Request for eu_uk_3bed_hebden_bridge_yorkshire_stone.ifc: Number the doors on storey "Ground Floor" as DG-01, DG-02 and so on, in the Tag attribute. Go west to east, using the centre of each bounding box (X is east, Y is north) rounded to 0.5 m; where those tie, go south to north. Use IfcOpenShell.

First a look at what the model holds.

```python
import ifcopenshell
import ifcopenshell.util.element
import ifcopenshell.util.placement

model = ifcopenshell.open("eu_uk_3bed_hebden_bridge_yorkshire_stone.ifc")
print(model.schema)
storey = next(s for s in model.by_type("IfcBuildingStorey") if s.Name == "Ground Floor")
doors = [e for e in ifcopenshell.util.element.get_decomposition(storey) if e.is_a("IfcDoor")]
for e in sorted(doors, key=lambda e: e.id()):
    origin = ifcopenshell.util.placement.get_local_placement(e.ObjectPlacement)[:3, 3]
    print(e.id(), e.Tag, e.Name, origin.round(2) + 0.0, sep=" | ")
```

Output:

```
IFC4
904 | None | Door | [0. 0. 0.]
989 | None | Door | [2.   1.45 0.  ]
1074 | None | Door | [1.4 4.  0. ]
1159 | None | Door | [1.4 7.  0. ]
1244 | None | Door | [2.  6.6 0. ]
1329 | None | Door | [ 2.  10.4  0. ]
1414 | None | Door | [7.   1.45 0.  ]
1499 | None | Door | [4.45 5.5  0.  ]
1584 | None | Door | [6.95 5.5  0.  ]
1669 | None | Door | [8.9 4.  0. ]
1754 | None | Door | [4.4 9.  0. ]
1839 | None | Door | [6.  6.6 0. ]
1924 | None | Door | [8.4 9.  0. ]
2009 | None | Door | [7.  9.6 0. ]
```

```python
import ifcopenshell
import ifcopenshell.geom
import ifcopenshell.util.element
import ifcopenshell.util.shape

model = ifcopenshell.open("eu_uk_3bed_hebden_bridge_yorkshire_stone.ifc")
settings = ifcopenshell.geom.settings()
settings.set("use-world-coords", True)


def centre(element):
    shape = ifcopenshell.geom.create_shape(settings, element)
    return ifcopenshell.util.shape.get_bbox_centroid(shape.geometry)


storey = next(s for s in model.by_type("IfcBuildingStorey") if s.Name == "Ground Floor")
doors = [e for e in ifcopenshell.util.element.get_decomposition(storey) if e.is_a("IfcDoor")]

# Insertion points can sit at a corner or the storey origin, so sort by the geometry (in metres).
centres = {e: centre(e) for e in doors}
doors.sort(key=lambda e: (round(centres[e][0] / 0.5), centres[e][1]))

for i, e in enumerate(doors, start=1):
    number = f"DG-{i:02d}"
    e.Tag = number
    print(e.id(), number)

model.write("eu_uk_3bed_hebden_bridge_yorkshire_stone_updated.ifc")
```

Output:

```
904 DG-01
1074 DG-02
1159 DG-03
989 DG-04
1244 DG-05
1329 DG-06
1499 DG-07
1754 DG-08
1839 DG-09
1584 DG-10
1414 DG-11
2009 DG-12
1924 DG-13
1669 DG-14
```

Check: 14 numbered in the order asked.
